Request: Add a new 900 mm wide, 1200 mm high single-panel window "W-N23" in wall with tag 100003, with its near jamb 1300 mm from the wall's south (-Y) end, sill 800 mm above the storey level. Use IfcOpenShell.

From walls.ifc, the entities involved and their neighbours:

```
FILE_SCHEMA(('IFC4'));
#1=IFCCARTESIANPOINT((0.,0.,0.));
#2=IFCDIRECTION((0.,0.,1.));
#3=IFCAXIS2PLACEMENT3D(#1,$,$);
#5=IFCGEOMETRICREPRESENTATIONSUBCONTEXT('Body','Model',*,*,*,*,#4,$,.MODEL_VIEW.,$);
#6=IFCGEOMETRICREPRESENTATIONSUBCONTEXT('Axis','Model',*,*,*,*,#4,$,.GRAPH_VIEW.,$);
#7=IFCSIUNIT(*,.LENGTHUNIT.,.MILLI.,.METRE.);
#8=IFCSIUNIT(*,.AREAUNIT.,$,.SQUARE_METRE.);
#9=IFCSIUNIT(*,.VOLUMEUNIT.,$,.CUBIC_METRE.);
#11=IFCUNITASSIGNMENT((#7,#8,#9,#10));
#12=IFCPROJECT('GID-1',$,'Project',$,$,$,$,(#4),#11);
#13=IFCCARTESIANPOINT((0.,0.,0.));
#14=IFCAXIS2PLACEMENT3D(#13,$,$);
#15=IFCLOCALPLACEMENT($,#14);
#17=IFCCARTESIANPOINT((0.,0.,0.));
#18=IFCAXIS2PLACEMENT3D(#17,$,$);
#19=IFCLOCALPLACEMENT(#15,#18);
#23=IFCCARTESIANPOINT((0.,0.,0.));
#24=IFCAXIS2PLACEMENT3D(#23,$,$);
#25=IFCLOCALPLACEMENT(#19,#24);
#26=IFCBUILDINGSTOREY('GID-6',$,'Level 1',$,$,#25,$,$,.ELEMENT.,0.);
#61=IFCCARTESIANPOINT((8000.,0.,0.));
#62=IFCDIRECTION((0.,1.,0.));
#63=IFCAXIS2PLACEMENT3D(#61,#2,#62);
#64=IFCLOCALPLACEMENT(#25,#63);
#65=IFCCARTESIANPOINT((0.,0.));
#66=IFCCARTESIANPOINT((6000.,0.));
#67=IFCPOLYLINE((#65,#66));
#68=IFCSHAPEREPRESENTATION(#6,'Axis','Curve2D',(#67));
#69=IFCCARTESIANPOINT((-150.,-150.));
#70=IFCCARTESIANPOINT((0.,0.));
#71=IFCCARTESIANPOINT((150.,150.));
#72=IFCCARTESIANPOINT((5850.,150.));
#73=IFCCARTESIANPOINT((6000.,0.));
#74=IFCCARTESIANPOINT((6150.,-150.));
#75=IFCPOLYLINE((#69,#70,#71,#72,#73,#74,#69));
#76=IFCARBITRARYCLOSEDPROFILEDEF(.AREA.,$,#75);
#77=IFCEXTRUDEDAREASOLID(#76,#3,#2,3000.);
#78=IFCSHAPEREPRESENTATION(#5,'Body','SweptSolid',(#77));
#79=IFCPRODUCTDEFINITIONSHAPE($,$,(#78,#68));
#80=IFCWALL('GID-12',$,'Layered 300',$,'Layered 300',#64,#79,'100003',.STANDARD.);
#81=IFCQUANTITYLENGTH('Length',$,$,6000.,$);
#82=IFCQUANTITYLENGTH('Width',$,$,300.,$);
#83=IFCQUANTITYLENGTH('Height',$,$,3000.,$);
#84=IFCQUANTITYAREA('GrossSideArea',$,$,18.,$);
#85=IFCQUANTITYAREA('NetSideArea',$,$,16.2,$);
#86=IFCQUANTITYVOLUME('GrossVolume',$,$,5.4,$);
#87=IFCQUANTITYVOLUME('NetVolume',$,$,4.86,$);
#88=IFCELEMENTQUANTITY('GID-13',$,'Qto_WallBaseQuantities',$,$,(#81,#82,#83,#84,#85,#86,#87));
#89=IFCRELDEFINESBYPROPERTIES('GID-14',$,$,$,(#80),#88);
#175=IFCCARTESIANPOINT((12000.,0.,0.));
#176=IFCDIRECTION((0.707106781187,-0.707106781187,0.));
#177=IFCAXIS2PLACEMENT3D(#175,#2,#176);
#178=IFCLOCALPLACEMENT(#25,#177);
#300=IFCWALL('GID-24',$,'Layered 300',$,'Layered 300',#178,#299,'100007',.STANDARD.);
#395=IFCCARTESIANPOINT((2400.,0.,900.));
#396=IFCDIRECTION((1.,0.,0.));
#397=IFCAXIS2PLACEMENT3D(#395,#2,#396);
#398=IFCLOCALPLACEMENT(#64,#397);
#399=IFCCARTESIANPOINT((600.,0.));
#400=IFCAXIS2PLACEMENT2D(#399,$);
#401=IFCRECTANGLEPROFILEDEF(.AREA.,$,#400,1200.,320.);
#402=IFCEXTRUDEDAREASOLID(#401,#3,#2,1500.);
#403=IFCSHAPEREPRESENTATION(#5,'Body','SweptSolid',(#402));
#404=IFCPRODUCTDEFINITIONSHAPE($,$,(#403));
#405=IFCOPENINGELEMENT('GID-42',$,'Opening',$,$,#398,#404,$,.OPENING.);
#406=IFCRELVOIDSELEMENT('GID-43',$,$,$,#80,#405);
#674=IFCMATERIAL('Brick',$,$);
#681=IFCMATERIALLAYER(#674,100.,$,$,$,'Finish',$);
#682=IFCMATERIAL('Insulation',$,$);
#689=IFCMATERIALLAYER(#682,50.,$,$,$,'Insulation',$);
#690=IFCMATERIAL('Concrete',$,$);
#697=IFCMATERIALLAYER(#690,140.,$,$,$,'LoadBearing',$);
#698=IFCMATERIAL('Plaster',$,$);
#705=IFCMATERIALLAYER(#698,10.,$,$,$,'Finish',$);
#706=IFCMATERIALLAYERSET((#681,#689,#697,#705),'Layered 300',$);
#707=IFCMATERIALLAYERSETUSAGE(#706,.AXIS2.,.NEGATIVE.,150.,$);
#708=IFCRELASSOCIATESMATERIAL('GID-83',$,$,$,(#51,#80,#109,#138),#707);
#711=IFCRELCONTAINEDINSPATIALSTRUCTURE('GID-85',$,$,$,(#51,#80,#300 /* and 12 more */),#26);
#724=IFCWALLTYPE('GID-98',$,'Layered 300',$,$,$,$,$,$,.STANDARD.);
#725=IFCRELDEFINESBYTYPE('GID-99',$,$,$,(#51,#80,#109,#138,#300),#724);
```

```python
import numpy as np
import ifcopenshell
import ifcopenshell.api.feature
import ifcopenshell.api.geometry
import ifcopenshell.api.pset
import ifcopenshell.api.root
import ifcopenshell.api.spatial
import ifcopenshell.geom
import ifcopenshell.util.element
import ifcopenshell.util.placement
import ifcopenshell.util.representation
import ifcopenshell.util.shape
import ifcopenshell.util.unit

model = ifcopenshell.open("walls.ifc")
unit_scale = ifcopenshell.util.unit.calculate_unit_scale(model)
area_scale = ifcopenshell.util.unit.calculate_unit_scale(model, "AREAUNIT")
volume_scale = ifcopenshell.util.unit.calculate_unit_scale(model, "VOLUMEUNIT")
settings = ifcopenshell.geom.settings()


def volume(element):
    """Net volume in cubic metres, openings subtracted."""
    shape = ifcopenshell.geom.create_shape(settings, element)
    return ifcopenshell.util.shape.get_volume(shape.geometry)


wall = model.by_guid("GID-12")
storey = ifcopenshell.util.element.get_container(wall, ifc_class="IfcBuildingStorey")
context = ifcopenshell.util.representation.get_context(model, "Model", "Body", "MODEL_VIEW")
before = volume(wall)

width, height, from_end, sill = 0.9, 1.2, 1.3, 0.8  # metres

# The wall runs along its own X axis, and the end named is its -X end.
wall_shape = ifcopenshell.geom.create_shape(settings, wall)
x, y, z = ifcopenshell.util.shape.get_vertices(wall_shape.geometry).T
start = x.min() + from_end
face, thickness = float(y.min()), float(y.max() - y.min())
wall_matrix = ifcopenshell.util.placement.get_local_placement(wall.ObjectPlacement)
level = ifcopenshell.util.placement.get_local_placement(storey.ObjectPlacement)[2, 3]


def in_wall(x, y):
    """Placement at x, y metres in the wall's axes, at sill height."""
    matrix = wall_matrix.copy()
    matrix[:, 3] = wall_matrix @ np.array([x / unit_scale, y / unit_scale, 0.0, 1.0])
    matrix[2, 3] = level + sill / unit_scale
    return matrix


# Opening: a box that overshoots both wall faces by 50 mm.
opening = ifcopenshell.api.root.create_entity(model, ifc_class="IfcOpeningElement", predefined_type="OPENING")
box = ifcopenshell.api.geometry.add_wall_representation(
    model, context=context, length=width, height=height, thickness=thickness + 0.1
)
ifcopenshell.api.geometry.assign_representation(model, product=opening, representation=box)
ifcopenshell.api.geometry.edit_object_placement(model, product=opening, matrix=in_wall(start, face - 0.05), is_si=False)
ifcopenshell.api.feature.add_feature(model, feature=opening, element=wall)

window = ifcopenshell.api.root.create_entity(model, ifc_class="IfcWindow", name="W-N23", predefined_type="WINDOW")
window.OverallWidth, window.OverallHeight = width / unit_scale, height / unit_scale
window.PartitioningType = "SINGLE_PANEL"
body = ifcopenshell.api.geometry.add_window_representation(
    model,
    context=context,
    overall_width=window.OverallWidth,
    overall_height=window.OverallHeight,
    partition_type="SINGLE_PANEL",
)
ifcopenshell.api.geometry.assign_representation(model, product=window, representation=body)
ifcopenshell.api.spatial.assign_container(model, products=[window], relating_structure=storey)
ifcopenshell.api.feature.add_filling(model, opening=opening, element=window)

# Centre the window in the wall's thickness.
ifcopenshell.api.geometry.edit_object_placement(model, product=window, matrix=in_wall(start, face), is_si=False)
window_shape = ifcopenshell.geom.create_shape(settings, window)
depth = ifcopenshell.util.shape.get_vertices(window_shape.geometry)[:, 1]
offset = face + thickness / 2 - (depth.min() + depth.max()) / 2
ifcopenshell.api.geometry.edit_object_placement(model, product=window, matrix=in_wall(start, offset), is_si=False)

after = volume(wall)

# Update the wall's stored quantities.
qto = model.by_id(ifcopenshell.util.element.get_pset(wall, "Qto_WallBaseQuantities", should_inherit=False)["id"])
ifcopenshell.api.pset.edit_qto(model, qto=qto, properties={
    "NetSideArea": after / thickness / area_scale,
    "NetVolume": after / volume_scale,
})

print(f"wall volume {before:.3f} -> {after:.3f} m3")

model.write("walls-out.ifc")
```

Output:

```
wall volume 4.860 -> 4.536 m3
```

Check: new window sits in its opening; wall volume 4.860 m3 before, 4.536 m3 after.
